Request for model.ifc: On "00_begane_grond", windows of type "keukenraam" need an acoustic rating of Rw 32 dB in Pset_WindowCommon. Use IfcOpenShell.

First a look at what the model holds.

```python
import ifcopenshell
import ifcopenshell.util.element

model = ifcopenshell.open("model.ifc")
print(model.schema)
storey = next(s for s in model.by_type("IfcBuildingStorey") if s.Name == "00_begane_grond")
windows = [e for e in ifcopenshell.util.element.get_decomposition(storey) if e.is_a("IfcWindow")]
seen = {}
for e in windows:
    element_type = ifcopenshell.util.element.get_type(e)
    key = (element_type.Name if element_type != e and element_type else None, ifcopenshell.util.element.get_pset(e, "Pset_WindowCommon", "AcousticRating"))
    seen[key] = seen.get(key, 0) + 1
for (name, value), count in sorted(seen.items(), key=str):
    print(count, "x", name, "|", value)
```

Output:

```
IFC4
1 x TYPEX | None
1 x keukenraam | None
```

```python
import ifcopenshell
import ifcopenshell.api.pset
import ifcopenshell.util.element

model = ifcopenshell.open("model.ifc")

storey = next(s for s in model.by_type("IfcBuildingStorey") if s.Name == "00_begane_grond")
windows = [e for e in ifcopenshell.util.element.get_decomposition(storey) if e.is_a("IfcWindow")]

count = 0
for e in windows:
    element_type = ifcopenshell.util.element.get_type(e)
    if element_type in (None, e) or element_type.Name != "keukenraam":
        continue
    # add_pset returns the element's existing set when there is one.
    pset = ifcopenshell.api.pset.add_pset(model, product=e, name="Pset_WindowCommon")
    ifcopenshell.api.pset.edit_pset(model, pset=pset, properties={"AcousticRating": "Rw 32 dB"})
    count += 1

print(count, "windows updated")

model.write("model_updated.ifc")
```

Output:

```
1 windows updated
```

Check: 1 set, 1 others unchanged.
